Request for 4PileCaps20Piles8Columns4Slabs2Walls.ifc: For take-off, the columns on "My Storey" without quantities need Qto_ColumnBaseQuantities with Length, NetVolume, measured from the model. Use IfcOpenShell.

First a look at what the model holds.

```python
import ifcopenshell
import ifcopenshell.util.element
import ifcopenshell.util.unit

model = ifcopenshell.open("4PileCaps20Piles8Columns4Slabs2Walls.ifc")
print(model.schema)
for unit_type in ("LENGTHUNIT", "AREAUNIT", "VOLUMEUNIT"):
    print(unit_type, ifcopenshell.util.unit.calculate_unit_scale(model, unit_type))
storey = next(s for s in model.by_type("IfcBuildingStorey") if s.Name == "My Storey")
columns = [e for e in ifcopenshell.util.element.get_decomposition(storey) if e.is_a("IfcColumn")]
for e in sorted(columns, key=lambda e: e.id()):
    print(e.id(), e.is_a(), e.Name, list(ifcopenshell.util.element.get_psets(e, qtos_only=True)), sep=" | ")
```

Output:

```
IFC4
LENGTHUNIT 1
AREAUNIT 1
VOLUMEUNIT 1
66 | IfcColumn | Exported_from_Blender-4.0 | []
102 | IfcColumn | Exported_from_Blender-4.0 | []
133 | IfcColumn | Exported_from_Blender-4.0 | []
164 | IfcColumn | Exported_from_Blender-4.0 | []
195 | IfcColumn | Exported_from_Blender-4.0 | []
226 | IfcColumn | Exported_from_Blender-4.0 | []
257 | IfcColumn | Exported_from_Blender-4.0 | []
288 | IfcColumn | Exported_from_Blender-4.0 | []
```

```python
import ifcopenshell
import ifcopenshell.api.pset
import ifcopenshell.geom
import ifcopenshell.util.element
import ifcopenshell.util.shape
import ifcopenshell.util.unit

model = ifcopenshell.open("4PileCaps20Piles8Columns4Slabs2Walls.ifc")
unit_scale = ifcopenshell.util.unit.calculate_unit_scale(model)
volume_scale = ifcopenshell.util.unit.calculate_unit_scale(model, "VOLUMEUNIT")
settings = ifcopenshell.geom.settings()

storey = next(s for s in model.by_type("IfcBuildingStorey") if s.Name == "My Storey")
columns = [e for e in ifcopenshell.util.element.get_decomposition(storey) if e.is_a("IfcColumn")]

for e in sorted(columns, key=lambda e: e.id()):
    if ifcopenshell.util.element.get_psets(e, qtos_only=True, should_inherit=False):
        continue
    # Geometry comes back in metres, in the element's own axes.
    shape = ifcopenshell.geom.create_shape(settings, e)
    values = {
        "Length": ifcopenshell.util.shape.get_z(shape.geometry) / unit_scale,
        "NetVolume": ifcopenshell.util.shape.get_volume(shape.geometry) / volume_scale,
    }
    qto = ifcopenshell.api.pset.add_qto(model, product=e, name="Qto_ColumnBaseQuantities")
    ifcopenshell.api.pset.edit_qto(model, qto=qto, properties=values)
    print(e.id(), {k: round(v, 3) for k, v in values.items()})

model.write("4PileCaps20Piles8Columns4Slabs2Walls-out.ifc")
```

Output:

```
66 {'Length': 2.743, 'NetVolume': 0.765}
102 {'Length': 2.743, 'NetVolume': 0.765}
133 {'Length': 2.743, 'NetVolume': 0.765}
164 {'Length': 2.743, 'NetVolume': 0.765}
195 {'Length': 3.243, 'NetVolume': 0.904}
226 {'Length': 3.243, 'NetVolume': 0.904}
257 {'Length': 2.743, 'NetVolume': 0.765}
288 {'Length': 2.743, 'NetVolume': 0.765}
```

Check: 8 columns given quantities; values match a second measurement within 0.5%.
